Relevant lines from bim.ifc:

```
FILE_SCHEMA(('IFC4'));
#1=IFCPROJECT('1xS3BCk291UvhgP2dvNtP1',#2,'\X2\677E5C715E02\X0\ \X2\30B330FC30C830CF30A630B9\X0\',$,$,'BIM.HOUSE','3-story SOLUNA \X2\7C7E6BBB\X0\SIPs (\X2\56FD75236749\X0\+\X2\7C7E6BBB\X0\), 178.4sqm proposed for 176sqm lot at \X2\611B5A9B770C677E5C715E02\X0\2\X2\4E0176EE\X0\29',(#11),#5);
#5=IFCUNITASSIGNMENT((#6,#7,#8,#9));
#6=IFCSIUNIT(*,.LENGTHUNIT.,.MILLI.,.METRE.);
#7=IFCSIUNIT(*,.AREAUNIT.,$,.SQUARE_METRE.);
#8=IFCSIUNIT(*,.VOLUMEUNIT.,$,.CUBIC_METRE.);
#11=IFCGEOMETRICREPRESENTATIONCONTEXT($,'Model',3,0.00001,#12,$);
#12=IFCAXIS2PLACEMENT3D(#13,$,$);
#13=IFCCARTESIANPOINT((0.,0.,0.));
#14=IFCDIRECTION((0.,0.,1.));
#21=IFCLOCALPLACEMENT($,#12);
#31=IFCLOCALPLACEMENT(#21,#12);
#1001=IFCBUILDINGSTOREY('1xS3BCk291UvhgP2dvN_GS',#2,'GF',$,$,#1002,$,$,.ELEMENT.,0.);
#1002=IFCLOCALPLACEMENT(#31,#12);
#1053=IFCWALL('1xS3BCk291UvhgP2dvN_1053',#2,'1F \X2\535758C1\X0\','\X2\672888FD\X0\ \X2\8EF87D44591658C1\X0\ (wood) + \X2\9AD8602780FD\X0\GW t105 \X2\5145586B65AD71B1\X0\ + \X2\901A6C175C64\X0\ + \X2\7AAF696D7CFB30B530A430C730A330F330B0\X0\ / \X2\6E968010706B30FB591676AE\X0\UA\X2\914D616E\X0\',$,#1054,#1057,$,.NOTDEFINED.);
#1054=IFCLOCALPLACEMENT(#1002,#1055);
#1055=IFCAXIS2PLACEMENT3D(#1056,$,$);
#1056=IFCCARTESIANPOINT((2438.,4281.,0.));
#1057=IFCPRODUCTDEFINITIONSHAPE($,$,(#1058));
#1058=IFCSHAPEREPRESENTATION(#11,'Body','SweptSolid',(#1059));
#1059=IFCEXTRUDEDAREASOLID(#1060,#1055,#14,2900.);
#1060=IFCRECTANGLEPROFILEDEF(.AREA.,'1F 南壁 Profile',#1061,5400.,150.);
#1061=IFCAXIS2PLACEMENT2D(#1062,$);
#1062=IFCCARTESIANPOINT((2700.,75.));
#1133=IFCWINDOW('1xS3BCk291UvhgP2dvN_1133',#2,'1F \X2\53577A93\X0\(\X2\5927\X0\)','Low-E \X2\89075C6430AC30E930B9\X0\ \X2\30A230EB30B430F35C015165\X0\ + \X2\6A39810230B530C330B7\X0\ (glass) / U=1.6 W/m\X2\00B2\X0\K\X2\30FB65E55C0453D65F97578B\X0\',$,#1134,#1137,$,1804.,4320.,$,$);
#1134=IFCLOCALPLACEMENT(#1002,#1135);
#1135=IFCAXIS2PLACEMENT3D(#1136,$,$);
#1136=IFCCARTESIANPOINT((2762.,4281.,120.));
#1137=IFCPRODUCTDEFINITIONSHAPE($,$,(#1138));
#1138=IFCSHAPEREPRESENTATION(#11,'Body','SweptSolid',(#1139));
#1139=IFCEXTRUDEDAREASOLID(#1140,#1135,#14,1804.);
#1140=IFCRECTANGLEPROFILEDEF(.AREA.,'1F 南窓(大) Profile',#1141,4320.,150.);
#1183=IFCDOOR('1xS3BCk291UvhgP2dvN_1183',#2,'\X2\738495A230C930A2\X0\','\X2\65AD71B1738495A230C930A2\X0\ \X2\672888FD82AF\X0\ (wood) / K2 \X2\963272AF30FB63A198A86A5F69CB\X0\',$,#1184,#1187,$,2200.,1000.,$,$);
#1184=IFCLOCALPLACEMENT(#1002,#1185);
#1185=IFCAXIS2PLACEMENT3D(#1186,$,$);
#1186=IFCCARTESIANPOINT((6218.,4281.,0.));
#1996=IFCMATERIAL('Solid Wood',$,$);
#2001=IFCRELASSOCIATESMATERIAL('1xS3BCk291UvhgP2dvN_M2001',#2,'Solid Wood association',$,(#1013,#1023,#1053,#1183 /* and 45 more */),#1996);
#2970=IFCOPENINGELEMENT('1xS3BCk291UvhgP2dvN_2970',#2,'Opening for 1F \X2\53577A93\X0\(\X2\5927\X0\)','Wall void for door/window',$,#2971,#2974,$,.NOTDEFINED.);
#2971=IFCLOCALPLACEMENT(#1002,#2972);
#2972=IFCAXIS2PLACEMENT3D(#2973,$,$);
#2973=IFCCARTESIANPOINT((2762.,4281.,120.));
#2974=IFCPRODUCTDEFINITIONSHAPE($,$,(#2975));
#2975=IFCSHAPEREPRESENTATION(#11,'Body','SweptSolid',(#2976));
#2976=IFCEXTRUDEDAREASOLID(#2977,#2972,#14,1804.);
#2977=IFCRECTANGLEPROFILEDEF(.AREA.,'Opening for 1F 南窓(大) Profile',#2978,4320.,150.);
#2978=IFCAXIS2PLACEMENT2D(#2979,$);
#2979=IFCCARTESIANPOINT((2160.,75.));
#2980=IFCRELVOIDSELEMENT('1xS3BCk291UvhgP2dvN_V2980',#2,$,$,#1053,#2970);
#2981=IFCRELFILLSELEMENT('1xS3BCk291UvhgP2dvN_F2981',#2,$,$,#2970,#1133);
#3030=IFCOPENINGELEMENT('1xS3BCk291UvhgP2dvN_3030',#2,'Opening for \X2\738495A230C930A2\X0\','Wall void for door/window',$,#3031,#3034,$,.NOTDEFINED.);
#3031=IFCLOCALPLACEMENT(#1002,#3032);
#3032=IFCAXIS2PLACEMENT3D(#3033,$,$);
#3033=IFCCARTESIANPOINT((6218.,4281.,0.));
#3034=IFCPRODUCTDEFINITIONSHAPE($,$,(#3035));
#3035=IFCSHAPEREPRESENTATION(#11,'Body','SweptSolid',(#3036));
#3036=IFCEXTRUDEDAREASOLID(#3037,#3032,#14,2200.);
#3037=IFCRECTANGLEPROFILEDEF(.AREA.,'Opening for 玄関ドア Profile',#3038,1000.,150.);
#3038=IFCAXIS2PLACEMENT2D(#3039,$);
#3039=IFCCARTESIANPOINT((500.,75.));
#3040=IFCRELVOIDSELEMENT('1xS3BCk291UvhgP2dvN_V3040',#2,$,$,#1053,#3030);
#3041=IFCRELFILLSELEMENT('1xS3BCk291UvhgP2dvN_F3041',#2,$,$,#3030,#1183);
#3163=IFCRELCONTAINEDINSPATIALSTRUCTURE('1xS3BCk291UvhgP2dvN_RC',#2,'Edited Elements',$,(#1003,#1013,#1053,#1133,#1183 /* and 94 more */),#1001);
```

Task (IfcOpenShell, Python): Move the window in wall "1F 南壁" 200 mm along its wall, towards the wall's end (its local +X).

```python
import ifcopenshell
import ifcopenshell.api.geometry
import ifcopenshell.util.placement
import ifcopenshell.util.unit

model = ifcopenshell.open("bim.ifc")
unit_scale = ifcopenshell.util.unit.calculate_unit_scale(model)

window = model.by_id(1133)
opening = window.FillsVoids[0].RelatingOpeningElement
wall = opening.VoidsElements[0].RelatingBuildingElement

wall_matrix = ifcopenshell.util.placement.get_local_placement(wall.ObjectPlacement)
shift = wall_matrix[:3, 0] * 0.2 / unit_scale
before = ifcopenshell.util.placement.get_local_placement(window.ObjectPlacement)[:3, 3].copy()

# The window is not placed relative to its opening, so move both.
for product in (opening, window):
    matrix = ifcopenshell.util.placement.get_local_placement(product.ObjectPlacement)
    matrix[:3, 3] += shift
    ifcopenshell.api.geometry.edit_object_placement(model, product=product, matrix=matrix, is_si=False)

after = ifcopenshell.util.placement.get_local_placement(window.ObjectPlacement)[:3, 3]
print("window moved by", (after - before).round(3) + 0.0)

model.write("bim_updated.ifc")
```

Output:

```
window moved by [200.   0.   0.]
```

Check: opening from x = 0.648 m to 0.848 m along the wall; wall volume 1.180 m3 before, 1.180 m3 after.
